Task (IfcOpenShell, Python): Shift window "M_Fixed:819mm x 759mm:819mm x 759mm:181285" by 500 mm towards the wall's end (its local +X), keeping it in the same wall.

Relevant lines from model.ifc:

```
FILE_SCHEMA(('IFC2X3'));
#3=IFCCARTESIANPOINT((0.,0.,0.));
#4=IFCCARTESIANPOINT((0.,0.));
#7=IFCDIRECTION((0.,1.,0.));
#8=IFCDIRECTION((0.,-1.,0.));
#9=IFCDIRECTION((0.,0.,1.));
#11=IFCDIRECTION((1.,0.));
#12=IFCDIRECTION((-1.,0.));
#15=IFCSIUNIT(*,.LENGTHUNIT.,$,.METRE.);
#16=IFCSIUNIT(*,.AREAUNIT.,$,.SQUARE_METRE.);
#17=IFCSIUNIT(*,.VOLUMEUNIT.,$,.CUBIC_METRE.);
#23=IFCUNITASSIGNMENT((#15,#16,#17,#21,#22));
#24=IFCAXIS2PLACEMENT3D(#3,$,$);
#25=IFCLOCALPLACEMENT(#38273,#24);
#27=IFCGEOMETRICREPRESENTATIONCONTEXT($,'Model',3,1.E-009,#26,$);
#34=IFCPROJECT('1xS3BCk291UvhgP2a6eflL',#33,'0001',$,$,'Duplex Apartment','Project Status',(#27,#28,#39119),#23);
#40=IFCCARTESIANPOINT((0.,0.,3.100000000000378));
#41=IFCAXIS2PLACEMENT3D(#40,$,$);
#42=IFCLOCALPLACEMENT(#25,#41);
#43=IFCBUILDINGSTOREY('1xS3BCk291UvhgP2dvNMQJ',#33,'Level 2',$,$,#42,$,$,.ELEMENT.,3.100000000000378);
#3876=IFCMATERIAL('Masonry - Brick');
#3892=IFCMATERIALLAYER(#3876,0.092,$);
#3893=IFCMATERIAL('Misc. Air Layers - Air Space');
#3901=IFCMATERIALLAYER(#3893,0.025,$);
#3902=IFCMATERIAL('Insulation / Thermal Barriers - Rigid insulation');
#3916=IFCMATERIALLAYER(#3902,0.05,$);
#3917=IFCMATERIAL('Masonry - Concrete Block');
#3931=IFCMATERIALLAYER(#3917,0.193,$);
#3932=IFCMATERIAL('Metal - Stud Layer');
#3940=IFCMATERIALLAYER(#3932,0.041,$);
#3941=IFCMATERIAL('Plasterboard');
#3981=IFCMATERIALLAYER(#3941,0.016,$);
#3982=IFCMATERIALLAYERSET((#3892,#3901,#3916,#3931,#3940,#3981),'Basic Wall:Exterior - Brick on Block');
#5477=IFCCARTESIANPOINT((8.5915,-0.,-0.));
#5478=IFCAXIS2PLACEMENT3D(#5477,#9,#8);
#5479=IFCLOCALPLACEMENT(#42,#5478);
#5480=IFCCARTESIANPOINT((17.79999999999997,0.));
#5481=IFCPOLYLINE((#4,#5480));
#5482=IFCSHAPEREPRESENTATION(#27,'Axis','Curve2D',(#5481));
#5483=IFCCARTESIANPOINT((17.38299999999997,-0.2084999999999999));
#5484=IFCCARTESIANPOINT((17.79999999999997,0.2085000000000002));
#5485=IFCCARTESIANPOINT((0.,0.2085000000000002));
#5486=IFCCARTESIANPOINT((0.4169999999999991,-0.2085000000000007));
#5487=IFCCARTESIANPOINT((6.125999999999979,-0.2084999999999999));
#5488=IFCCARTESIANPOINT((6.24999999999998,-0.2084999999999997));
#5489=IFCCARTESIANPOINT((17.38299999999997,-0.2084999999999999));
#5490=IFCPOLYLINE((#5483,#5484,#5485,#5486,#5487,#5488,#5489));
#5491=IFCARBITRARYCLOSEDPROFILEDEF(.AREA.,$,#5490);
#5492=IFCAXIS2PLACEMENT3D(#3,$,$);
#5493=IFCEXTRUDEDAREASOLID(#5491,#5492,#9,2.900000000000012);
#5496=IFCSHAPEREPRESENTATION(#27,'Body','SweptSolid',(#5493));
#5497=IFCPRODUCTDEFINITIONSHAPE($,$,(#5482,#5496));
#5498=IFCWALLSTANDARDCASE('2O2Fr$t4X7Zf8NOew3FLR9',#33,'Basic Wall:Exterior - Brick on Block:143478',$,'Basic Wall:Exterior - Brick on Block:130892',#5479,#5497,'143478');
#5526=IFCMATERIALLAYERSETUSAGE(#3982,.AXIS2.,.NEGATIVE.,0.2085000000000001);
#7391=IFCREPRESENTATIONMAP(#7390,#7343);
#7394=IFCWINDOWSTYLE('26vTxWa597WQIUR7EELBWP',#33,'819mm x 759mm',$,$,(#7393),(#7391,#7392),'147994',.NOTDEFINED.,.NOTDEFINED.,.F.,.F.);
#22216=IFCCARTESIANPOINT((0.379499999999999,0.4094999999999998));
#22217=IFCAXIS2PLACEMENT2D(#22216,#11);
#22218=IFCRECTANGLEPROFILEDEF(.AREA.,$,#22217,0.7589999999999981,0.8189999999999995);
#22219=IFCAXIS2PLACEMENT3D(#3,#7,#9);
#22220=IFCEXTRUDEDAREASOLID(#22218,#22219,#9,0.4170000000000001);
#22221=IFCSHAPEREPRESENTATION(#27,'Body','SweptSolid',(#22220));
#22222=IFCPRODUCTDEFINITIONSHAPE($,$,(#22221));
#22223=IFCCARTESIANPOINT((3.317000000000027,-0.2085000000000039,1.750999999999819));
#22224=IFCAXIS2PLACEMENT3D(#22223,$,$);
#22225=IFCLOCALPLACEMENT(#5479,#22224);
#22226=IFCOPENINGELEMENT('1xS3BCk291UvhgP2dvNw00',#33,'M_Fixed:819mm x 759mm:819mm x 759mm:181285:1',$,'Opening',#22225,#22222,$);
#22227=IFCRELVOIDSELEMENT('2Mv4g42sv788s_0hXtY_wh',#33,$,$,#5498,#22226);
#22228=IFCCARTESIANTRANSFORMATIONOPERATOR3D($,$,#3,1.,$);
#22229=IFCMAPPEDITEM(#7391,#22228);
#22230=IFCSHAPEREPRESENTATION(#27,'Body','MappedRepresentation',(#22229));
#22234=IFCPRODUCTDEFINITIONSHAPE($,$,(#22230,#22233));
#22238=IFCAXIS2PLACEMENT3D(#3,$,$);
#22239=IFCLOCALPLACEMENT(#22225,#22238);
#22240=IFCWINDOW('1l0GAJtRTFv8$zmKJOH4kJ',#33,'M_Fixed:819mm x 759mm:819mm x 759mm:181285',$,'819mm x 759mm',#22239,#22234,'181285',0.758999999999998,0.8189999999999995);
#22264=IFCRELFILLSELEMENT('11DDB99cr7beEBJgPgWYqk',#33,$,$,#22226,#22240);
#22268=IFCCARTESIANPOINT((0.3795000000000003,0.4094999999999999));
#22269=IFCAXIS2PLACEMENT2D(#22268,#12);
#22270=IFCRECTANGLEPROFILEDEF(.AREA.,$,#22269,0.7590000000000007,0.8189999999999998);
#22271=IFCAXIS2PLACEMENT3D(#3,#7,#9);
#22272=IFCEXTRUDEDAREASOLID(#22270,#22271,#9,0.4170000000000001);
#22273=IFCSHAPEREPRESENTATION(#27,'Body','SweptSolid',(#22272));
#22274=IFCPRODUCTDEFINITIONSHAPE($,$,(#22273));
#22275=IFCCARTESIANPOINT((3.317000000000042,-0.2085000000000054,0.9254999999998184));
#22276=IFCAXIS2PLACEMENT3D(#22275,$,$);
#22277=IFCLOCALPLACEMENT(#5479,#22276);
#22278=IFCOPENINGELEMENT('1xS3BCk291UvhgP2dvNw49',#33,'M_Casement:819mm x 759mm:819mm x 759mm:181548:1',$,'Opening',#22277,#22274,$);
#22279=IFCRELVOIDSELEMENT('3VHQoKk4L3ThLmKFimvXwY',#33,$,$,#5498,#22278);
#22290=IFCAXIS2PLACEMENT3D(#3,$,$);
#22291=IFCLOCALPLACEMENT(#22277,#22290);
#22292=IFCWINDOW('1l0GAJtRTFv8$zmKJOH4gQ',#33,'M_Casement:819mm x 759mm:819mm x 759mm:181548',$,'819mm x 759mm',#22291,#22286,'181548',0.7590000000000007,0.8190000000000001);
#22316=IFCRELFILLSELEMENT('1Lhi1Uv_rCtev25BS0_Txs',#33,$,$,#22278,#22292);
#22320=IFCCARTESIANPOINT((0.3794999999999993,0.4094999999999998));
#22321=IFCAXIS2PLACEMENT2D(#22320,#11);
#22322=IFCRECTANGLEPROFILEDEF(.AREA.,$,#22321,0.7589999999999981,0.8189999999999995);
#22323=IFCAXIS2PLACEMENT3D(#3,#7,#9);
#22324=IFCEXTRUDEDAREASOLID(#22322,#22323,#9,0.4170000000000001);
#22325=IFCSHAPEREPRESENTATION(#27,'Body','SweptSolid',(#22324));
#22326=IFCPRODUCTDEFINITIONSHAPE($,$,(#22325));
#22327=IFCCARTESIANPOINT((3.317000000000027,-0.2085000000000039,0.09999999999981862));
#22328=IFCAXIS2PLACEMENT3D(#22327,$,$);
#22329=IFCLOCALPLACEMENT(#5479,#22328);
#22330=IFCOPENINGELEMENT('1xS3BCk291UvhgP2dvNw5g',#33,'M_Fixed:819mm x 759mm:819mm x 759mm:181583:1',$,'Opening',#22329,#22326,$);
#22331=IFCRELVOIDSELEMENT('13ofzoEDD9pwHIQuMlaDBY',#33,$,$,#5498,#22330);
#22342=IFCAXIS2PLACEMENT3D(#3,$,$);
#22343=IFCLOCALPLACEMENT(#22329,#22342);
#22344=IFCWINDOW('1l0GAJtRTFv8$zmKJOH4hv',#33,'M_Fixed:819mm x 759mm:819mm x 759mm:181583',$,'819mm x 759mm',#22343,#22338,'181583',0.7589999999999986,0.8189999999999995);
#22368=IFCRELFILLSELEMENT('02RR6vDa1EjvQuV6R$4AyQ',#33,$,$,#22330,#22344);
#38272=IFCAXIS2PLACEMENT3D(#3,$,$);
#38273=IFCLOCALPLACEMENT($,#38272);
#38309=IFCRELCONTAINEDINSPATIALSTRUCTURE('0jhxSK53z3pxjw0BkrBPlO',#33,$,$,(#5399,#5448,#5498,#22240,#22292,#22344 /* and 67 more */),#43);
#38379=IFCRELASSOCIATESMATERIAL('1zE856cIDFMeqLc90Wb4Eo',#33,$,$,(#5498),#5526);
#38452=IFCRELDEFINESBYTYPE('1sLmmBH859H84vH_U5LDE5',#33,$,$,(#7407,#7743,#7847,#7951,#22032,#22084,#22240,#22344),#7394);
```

```python
import ifcopenshell
import ifcopenshell.api.geometry
import ifcopenshell.util.placement
import ifcopenshell.util.unit

model = ifcopenshell.open("model.ifc")
unit_scale = ifcopenshell.util.unit.calculate_unit_scale(model)

window = model.by_id(22240)
opening = window.FillsVoids[0].RelatingOpeningElement
wall = opening.VoidsElements[0].RelatingBuildingElement

wall_matrix = ifcopenshell.util.placement.get_local_placement(wall.ObjectPlacement)
shift = wall_matrix[:3, 0] * 0.5 / unit_scale
before = ifcopenshell.util.placement.get_local_placement(window.ObjectPlacement)[:3, 3].copy()

# The window is placed relative to its opening, so it follows when the opening moves.
matrix = ifcopenshell.util.placement.get_local_placement(opening.ObjectPlacement)
matrix[:3, 3] += shift
ifcopenshell.api.geometry.edit_object_placement(
    model, product=opening, matrix=matrix, is_si=False, should_transform_children=True
)

after = ifcopenshell.util.placement.get_local_placement(window.ObjectPlacement)[:3, 3]
print("window moved by", (after - before).round(3) + 0.0)

model.write("model_updated.ifc")
```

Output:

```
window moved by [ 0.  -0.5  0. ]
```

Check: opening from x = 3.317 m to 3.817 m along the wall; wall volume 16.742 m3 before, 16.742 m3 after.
